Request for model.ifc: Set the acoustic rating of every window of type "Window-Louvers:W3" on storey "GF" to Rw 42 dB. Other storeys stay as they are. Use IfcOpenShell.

First a look at what the model holds.

```python
import ifcopenshell
import ifcopenshell.util.element

model = ifcopenshell.open("model.ifc")
print(model.schema)
storey = next(s for s in model.by_type("IfcBuildingStorey") if s.Name == "GF")
windows = [e for e in ifcopenshell.util.element.get_decomposition(storey) if e.is_a("IfcWindow")]
seen = {}
for e in windows:
    element_type = ifcopenshell.util.element.get_type(e)
    key = (element_type.Name if element_type != e and element_type else None, ifcopenshell.util.element.get_pset(e, "Pset_WindowCommon", "AcousticRating"))
    seen[key] = seen.get(key, 0) + 1
for (name, value), count in sorted(seen.items(), key=str):
    print(count, "x", name, "|", value)
```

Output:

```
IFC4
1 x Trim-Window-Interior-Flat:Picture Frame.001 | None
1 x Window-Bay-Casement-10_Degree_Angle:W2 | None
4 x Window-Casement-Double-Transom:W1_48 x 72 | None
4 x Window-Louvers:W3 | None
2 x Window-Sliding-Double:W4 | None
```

```python
import ifcopenshell
import ifcopenshell.api.pset
import ifcopenshell.util.element

model = ifcopenshell.open("model.ifc")

storey = next(s for s in model.by_type("IfcBuildingStorey") if s.Name == "GF")
windows = [e for e in ifcopenshell.util.element.get_decomposition(storey) if e.is_a("IfcWindow")]

count = 0
for e in windows:
    element_type = ifcopenshell.util.element.get_type(e)
    if element_type in (None, e) or element_type.Name != "Window-Louvers:W3":
        continue
    # add_pset returns the element's existing set when there is one.
    pset = ifcopenshell.api.pset.add_pset(model, product=e, name="Pset_WindowCommon")
    ifcopenshell.api.pset.edit_pset(model, pset=pset, properties={"AcousticRating": "Rw 42 dB"})
    count += 1

print(count, "windows updated")

model.write("model_rev.ifc")
```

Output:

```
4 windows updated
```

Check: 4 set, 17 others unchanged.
